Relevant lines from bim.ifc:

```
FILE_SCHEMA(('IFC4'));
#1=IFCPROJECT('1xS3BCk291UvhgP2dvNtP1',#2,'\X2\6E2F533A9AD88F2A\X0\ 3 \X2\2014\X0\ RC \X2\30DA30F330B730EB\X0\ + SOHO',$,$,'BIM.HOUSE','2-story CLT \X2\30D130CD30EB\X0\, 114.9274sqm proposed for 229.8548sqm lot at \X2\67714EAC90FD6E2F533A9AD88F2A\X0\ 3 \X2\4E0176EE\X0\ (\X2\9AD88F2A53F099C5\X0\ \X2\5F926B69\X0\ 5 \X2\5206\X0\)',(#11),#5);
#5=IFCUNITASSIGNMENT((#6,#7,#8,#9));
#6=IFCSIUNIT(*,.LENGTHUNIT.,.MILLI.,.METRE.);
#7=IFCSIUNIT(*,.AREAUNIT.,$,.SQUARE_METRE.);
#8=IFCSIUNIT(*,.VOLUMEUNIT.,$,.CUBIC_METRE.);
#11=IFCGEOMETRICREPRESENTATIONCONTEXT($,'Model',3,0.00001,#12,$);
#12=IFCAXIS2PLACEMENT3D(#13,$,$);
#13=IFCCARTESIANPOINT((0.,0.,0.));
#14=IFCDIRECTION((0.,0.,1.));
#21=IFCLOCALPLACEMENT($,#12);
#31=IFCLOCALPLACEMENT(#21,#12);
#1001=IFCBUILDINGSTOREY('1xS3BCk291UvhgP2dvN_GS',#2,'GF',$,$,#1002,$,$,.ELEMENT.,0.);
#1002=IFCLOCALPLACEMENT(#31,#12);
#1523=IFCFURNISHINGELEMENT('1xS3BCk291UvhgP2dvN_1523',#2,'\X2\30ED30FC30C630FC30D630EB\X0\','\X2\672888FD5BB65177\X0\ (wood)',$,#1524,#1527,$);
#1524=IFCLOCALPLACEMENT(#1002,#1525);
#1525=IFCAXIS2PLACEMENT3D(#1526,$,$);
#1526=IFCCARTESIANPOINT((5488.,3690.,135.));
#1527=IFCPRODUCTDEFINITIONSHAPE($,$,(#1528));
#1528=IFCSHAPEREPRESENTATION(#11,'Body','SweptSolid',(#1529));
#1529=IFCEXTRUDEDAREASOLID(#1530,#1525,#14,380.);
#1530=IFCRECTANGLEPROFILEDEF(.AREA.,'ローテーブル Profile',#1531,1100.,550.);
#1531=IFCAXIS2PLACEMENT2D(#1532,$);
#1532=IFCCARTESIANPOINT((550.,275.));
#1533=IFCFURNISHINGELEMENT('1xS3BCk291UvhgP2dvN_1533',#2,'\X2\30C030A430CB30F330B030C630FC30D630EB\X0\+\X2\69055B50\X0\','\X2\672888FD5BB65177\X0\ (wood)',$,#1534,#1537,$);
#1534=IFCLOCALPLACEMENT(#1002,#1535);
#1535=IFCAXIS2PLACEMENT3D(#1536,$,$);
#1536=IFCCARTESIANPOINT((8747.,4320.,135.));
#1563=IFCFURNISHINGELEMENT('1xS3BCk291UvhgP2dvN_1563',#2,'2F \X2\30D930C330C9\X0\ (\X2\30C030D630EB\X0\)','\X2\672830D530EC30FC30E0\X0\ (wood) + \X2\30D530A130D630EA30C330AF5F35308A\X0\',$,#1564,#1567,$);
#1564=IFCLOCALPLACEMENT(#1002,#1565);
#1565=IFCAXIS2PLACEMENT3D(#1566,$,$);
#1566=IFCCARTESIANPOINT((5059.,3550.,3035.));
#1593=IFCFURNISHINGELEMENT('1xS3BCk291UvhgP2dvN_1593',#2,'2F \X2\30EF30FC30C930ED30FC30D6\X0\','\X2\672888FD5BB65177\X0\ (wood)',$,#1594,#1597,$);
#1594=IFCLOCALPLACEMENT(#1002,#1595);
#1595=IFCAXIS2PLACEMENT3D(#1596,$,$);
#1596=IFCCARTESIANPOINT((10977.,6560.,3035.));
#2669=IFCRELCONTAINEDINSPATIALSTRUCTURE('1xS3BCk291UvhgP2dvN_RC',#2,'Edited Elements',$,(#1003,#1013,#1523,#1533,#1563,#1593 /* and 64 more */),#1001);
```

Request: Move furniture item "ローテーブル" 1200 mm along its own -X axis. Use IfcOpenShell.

```python
import ifcopenshell
import ifcopenshell.api.geometry
import ifcopenshell.util.placement
import ifcopenshell.util.unit

model = ifcopenshell.open("bim.ifc")
unit_scale = ifcopenshell.util.unit.calculate_unit_scale(model)

item = model.by_guid("1xS3BCk291UvhgP2dvN_1523")
matrix = ifcopenshell.util.placement.get_local_placement(item.ObjectPlacement)
matrix[:3, 3] -= matrix[:3, 0] * 1.2 / unit_scale
ifcopenshell.api.geometry.edit_object_placement(model, product=item, matrix=matrix, is_si=False)

print(ifcopenshell.util.placement.get_local_placement(item.ObjectPlacement).round(3) + 0.0)

model.write("bim_updated.ifc")
```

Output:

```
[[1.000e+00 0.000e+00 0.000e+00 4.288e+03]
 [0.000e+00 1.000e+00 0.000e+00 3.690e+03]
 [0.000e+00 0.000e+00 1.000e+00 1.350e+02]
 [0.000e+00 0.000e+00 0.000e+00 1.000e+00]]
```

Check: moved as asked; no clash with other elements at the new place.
